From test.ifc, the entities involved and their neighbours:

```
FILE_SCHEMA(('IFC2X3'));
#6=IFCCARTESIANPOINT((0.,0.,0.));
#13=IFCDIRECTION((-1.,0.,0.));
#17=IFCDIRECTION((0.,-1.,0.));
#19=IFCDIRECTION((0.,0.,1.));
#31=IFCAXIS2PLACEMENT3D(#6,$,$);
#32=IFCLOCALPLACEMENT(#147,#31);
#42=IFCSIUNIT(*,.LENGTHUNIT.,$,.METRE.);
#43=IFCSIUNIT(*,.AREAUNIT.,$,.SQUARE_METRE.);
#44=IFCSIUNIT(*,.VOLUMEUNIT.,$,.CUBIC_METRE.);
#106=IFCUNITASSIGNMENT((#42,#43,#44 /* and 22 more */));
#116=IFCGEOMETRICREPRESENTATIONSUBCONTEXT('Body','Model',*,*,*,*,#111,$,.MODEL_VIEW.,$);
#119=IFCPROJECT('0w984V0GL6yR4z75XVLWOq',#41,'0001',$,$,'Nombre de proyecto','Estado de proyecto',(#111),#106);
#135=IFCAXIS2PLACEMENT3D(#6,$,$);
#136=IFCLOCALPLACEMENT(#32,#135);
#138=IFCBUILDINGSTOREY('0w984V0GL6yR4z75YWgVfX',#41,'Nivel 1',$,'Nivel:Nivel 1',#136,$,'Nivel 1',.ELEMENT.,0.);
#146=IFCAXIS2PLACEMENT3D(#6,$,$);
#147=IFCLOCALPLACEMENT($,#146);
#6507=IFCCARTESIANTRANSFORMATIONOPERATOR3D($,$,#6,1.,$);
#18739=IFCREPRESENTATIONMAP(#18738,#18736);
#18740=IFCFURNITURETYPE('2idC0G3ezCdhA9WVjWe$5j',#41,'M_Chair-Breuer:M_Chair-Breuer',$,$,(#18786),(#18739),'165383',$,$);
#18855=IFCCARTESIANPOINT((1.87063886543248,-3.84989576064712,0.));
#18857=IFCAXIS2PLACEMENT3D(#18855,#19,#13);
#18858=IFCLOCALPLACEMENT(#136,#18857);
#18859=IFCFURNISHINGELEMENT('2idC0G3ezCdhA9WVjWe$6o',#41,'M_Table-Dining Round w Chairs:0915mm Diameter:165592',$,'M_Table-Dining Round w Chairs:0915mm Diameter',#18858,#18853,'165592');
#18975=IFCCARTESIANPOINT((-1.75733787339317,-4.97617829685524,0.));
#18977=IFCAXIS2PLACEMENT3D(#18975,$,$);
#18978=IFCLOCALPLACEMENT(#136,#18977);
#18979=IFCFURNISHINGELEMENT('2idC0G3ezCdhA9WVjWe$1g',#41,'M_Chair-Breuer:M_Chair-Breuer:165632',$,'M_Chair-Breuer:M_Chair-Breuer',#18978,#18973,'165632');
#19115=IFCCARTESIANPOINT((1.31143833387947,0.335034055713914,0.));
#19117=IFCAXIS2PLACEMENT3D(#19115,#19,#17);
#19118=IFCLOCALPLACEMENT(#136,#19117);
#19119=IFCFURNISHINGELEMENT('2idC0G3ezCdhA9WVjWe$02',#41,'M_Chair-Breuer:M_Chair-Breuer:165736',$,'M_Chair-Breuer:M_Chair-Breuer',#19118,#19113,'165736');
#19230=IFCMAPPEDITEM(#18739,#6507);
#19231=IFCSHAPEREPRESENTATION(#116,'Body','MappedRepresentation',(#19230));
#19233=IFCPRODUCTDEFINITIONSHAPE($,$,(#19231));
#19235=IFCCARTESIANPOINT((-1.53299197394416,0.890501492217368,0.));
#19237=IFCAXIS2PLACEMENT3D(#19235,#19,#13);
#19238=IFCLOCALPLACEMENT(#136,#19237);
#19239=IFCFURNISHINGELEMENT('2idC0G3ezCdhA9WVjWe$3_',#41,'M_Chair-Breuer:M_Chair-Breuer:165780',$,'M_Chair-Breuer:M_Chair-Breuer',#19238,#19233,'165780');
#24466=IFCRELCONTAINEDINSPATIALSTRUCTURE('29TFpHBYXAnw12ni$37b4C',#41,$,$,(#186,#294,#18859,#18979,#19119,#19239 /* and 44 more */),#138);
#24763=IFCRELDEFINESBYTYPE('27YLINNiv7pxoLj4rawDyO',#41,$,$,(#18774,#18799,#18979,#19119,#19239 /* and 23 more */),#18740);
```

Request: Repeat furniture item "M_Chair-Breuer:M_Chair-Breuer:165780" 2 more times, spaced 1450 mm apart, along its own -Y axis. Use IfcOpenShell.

```python
import ifcopenshell
import ifcopenshell.api.geometry
import ifcopenshell.api.root
import ifcopenshell.util.element
import ifcopenshell.util.placement

model = ifcopenshell.open("test.ifc")


def reuse_history(source, copy):
    """copy_class also copies each property set's owner history, people and application; keep the originals."""
    for rel in copy.IsDefinedBy:
        if rel.is_a("IfcRelDefinesByProperties") and (history := rel.RelatingPropertyDefinition.OwnerHistory):
            rel.RelatingPropertyDefinition.OwnerHistory = source.OwnerHistory
            ifcopenshell.util.element.remove_deep2(model, history)


source = model.by_guid("2idC0G3ezCdhA9WVjWe$3_")
base = ifcopenshell.util.placement.get_local_placement(source.ObjectPlacement)
step = -base[:3, 1] * 1.45

for i in range(1, 3):
    copy = ifcopenshell.api.root.copy_class(model, product=source)
    copy.Representation = ifcopenshell.util.element.copy_deep(
        model, source.Representation, exclude=["IfcGeometricRepresentationContext", "IfcRepresentationMap"]
    )
    copy.Name = "M_Chair-Breuer:M_Chair-Breuer"
    copy.Tag = None
    reuse_history(source, copy)
    matrix = base.copy()
    matrix[:3, 3] += i * step
    print("added at", matrix[:3, 3].round(3) + 0.0)
    ifcopenshell.api.geometry.edit_object_placement(model, product=copy, matrix=matrix, is_si=False)

model.write("test_rev.ifc")
```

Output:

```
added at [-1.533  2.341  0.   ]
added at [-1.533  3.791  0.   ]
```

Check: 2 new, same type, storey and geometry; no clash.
